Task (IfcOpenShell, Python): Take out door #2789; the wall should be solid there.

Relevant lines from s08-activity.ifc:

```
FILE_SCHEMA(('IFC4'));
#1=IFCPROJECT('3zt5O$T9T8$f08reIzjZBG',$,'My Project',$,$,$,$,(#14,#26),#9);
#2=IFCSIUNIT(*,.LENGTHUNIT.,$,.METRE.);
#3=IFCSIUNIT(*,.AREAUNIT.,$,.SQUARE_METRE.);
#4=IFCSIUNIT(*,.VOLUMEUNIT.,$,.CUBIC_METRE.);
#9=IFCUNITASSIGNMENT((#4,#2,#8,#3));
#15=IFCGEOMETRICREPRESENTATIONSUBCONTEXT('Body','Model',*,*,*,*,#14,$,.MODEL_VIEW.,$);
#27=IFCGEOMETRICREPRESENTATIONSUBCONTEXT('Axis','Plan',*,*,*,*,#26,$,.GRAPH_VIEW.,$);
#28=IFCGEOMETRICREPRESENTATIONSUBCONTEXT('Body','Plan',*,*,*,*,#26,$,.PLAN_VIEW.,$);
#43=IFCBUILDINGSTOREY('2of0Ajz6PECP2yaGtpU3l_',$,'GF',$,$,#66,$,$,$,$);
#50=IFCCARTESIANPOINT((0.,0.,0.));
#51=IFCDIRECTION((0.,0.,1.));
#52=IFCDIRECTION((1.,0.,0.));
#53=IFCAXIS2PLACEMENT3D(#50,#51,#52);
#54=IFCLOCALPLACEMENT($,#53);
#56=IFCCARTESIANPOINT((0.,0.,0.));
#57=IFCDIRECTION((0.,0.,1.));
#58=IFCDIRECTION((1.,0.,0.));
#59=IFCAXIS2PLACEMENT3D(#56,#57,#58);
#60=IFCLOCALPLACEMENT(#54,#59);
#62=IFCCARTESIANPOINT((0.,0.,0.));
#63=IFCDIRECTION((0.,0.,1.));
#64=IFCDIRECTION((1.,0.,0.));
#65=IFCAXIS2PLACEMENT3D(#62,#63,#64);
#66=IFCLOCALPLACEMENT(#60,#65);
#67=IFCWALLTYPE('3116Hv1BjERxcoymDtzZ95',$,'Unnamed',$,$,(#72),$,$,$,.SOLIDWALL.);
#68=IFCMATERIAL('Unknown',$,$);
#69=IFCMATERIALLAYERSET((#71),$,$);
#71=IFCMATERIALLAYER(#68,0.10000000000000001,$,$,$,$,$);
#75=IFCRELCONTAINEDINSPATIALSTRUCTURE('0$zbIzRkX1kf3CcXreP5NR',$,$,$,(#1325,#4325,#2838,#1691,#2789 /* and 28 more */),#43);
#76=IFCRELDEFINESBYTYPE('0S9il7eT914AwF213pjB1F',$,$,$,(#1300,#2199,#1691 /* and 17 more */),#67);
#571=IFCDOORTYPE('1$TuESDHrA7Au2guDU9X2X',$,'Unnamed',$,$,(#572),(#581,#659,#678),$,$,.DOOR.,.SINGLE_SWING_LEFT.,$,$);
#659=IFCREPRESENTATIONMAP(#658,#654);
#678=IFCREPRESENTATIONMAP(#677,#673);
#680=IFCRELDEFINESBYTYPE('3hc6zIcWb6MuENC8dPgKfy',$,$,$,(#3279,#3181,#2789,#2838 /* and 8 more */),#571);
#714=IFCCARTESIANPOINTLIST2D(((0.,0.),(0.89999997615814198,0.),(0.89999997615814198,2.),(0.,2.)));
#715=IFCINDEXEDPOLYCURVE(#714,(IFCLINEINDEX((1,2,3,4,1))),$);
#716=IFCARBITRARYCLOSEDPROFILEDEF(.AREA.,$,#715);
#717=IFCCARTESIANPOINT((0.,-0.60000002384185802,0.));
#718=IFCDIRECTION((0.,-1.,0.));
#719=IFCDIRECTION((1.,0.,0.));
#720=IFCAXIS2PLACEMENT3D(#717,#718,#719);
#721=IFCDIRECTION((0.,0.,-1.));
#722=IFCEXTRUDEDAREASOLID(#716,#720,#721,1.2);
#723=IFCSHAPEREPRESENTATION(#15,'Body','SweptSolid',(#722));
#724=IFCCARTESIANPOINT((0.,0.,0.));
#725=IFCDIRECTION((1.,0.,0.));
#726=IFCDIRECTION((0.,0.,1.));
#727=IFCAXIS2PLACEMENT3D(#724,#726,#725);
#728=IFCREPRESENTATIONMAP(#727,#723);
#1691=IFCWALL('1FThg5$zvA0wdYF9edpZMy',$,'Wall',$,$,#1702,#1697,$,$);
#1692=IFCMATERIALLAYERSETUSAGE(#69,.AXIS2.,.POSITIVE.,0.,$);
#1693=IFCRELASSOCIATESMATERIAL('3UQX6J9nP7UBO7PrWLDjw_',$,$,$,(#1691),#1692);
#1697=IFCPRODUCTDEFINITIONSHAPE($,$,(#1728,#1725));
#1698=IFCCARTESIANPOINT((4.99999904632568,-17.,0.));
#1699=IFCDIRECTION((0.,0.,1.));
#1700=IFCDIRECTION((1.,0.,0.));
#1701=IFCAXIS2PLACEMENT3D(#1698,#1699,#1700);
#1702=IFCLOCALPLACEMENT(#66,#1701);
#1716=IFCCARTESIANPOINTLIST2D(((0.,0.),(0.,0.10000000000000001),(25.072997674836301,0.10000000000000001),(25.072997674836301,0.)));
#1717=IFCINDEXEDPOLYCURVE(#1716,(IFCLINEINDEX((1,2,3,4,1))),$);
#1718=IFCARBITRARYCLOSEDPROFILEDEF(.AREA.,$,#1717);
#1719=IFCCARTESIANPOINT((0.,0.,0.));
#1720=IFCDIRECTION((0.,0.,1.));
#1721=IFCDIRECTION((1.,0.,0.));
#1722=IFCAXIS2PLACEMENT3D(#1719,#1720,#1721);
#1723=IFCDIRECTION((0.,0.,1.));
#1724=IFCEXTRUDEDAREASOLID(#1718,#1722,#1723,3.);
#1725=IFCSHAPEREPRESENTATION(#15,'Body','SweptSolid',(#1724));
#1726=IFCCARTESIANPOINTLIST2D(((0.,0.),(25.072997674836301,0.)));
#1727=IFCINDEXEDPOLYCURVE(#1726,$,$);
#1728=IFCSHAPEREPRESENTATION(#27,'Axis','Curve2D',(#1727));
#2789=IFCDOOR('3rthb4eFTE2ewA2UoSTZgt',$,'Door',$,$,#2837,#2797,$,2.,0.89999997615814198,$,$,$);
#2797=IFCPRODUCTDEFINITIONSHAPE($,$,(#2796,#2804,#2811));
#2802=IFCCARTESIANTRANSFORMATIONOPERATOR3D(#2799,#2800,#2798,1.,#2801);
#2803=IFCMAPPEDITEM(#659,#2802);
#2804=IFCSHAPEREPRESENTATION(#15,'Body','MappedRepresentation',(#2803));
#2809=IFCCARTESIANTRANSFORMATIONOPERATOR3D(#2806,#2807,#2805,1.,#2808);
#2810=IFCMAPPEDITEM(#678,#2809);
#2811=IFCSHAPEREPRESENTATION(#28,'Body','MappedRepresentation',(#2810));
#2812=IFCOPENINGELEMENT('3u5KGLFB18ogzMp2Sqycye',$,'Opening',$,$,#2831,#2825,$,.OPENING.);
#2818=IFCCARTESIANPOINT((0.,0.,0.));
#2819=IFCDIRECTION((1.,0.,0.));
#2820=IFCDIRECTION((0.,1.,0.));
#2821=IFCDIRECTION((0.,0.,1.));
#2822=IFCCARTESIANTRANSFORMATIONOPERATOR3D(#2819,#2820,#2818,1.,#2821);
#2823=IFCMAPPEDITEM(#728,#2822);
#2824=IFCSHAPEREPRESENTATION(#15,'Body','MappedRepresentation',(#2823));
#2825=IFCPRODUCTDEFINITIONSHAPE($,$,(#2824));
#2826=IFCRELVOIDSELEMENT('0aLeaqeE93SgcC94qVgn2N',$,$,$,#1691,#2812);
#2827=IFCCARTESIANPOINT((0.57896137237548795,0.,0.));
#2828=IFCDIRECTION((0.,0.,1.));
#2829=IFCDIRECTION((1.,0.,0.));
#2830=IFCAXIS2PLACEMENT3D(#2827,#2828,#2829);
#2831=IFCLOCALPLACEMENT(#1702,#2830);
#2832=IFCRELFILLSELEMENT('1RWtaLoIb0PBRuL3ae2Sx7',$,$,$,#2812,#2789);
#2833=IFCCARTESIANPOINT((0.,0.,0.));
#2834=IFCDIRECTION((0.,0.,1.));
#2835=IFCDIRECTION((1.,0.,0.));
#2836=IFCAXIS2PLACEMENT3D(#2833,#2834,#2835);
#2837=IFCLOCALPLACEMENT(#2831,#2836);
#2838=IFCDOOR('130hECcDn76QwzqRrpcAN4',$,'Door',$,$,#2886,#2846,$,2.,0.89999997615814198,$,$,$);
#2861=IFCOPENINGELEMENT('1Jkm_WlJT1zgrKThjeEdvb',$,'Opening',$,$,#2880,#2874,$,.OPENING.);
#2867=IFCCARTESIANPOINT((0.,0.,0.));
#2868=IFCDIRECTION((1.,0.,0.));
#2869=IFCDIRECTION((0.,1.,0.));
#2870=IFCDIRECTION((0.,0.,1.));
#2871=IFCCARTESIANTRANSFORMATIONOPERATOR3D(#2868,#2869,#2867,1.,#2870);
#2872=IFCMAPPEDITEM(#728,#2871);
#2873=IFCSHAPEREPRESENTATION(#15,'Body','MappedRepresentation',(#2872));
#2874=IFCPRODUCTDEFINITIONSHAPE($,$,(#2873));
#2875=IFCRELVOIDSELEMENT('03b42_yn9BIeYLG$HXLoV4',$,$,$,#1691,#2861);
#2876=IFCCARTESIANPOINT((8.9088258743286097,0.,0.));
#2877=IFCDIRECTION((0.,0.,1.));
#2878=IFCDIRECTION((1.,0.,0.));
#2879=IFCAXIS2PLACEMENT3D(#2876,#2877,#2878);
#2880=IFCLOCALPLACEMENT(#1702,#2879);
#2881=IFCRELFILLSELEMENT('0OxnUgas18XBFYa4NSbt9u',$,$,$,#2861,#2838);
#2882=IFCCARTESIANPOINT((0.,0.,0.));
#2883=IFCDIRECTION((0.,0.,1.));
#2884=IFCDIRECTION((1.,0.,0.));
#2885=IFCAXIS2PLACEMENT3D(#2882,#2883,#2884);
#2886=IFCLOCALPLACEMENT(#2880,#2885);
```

```python
import ifcopenshell
import ifcopenshell.api.feature
import ifcopenshell.api.root
import ifcopenshell.geom
import ifcopenshell.util.shape

model = ifcopenshell.open("s08-activity.ifc")
settings = ifcopenshell.geom.settings()


def volume(element):
    """Net volume in cubic metres, openings subtracted."""
    shape = ifcopenshell.geom.create_shape(settings, element)
    return ifcopenshell.util.shape.get_volume(shape.geometry)


door = model.by_guid("3rthb4eFTE2ewA2UoSTZgt")
opening = door.FillsVoids[0].RelatingOpeningElement
wall = opening.VoidsElements[0].RelatingBuildingElement
before = volume(wall)

ifcopenshell.api.root.remove_product(model, product=door)
ifcopenshell.api.feature.remove_feature(model, feature=opening)

after = volume(wall)

print(f"wall volume {before:.3f} -> {after:.3f} m3")

model.write("s08-activity_v2.ifc")
```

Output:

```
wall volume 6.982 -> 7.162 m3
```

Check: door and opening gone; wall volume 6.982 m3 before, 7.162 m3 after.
